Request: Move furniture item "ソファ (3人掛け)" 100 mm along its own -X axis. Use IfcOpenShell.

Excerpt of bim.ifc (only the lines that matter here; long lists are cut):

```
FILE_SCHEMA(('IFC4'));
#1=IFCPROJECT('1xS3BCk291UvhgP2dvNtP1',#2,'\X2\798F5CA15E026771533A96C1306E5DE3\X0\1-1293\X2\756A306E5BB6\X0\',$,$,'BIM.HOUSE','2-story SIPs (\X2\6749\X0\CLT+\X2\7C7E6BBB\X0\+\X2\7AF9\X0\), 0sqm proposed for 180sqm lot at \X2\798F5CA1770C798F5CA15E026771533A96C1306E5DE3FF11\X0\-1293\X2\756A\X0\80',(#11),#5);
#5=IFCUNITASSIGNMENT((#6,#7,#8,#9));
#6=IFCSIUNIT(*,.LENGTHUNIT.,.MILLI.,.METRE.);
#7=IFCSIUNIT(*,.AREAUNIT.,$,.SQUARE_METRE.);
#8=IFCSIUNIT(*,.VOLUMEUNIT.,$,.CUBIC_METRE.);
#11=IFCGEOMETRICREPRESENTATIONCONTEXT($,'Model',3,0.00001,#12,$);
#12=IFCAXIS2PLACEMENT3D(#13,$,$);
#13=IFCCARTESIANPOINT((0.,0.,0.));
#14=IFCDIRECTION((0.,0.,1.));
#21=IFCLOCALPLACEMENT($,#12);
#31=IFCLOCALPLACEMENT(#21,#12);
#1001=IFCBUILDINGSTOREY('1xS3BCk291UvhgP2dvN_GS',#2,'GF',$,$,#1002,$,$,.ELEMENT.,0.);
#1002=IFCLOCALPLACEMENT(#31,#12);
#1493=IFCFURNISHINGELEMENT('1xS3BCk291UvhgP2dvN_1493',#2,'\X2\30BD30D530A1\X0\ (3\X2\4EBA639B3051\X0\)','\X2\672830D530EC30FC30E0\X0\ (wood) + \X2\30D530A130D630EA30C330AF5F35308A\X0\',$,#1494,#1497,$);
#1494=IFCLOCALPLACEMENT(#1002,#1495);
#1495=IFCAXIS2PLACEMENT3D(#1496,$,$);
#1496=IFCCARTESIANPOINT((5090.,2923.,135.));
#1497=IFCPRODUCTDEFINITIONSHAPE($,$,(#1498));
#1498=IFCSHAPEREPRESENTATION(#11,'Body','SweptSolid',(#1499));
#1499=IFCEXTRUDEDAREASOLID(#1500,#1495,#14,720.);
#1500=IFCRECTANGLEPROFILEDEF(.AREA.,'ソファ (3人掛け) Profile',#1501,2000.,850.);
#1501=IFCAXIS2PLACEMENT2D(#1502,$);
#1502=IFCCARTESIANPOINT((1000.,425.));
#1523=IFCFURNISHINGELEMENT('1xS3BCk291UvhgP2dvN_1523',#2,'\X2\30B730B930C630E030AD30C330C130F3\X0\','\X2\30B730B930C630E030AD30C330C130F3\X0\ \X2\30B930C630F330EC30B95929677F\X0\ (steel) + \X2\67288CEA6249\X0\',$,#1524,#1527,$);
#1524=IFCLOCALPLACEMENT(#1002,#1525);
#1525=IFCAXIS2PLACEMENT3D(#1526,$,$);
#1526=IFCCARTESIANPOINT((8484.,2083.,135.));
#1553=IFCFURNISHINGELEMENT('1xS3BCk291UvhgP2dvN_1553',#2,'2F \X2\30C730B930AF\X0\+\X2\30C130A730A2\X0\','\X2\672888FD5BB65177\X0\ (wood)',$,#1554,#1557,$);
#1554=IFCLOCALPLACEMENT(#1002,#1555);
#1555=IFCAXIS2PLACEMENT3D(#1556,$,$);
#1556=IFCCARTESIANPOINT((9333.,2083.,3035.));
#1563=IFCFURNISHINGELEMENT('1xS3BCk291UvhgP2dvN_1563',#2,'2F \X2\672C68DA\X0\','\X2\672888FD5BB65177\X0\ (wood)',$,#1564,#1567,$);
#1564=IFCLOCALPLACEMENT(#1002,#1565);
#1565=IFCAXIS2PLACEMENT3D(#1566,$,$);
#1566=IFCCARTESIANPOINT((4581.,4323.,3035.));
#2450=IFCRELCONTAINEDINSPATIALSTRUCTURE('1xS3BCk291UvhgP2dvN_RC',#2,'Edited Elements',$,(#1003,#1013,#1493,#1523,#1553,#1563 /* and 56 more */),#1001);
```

```python
import ifcopenshell
import ifcopenshell.api.geometry
import ifcopenshell.util.placement
import ifcopenshell.util.unit

model = ifcopenshell.open("bim.ifc")
unit_scale = ifcopenshell.util.unit.calculate_unit_scale(model)

item = model.by_guid("1xS3BCk291UvhgP2dvN_1493")
matrix = ifcopenshell.util.placement.get_local_placement(item.ObjectPlacement)
matrix[:3, 3] -= matrix[:3, 0] * 0.1 / unit_scale
ifcopenshell.api.geometry.edit_object_placement(model, product=item, matrix=matrix, is_si=False)

print(ifcopenshell.util.placement.get_local_placement(item.ObjectPlacement).round(3) + 0.0)

model.write("bim_updated.ifc")
```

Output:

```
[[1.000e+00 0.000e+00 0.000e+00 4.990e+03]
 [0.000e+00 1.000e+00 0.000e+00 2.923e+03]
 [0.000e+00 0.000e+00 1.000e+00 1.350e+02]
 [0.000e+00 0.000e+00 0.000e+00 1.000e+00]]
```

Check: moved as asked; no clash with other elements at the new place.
